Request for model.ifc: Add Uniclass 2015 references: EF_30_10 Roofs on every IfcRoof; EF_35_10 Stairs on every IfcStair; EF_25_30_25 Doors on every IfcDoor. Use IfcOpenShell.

First a look at what the model holds.

```python
import ifcopenshell

model = ifcopenshell.open("model.ifc")
print(model.schema)
print("classifications:", [c.Name for c in model.by_type("IfcClassification")])
for ifc_class in ("IfcDoor", "IfcRoof", "IfcStair", "IfcWall", "IfcWindow"):
    print(ifc_class, len(model.by_type(ifc_class)))
```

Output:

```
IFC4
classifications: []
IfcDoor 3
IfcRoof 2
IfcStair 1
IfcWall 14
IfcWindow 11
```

```python
import ifcopenshell
import ifcopenshell.api.classification

model = ifcopenshell.open("model.ifc")

system = ifcopenshell.api.classification.add_classification(model, classification="Uniclass 2015")

codes = {
    "IfcRoof": ("EF_30_10", "Roofs"),
    "IfcStair": ("EF_35_10", "Stairs"),
    "IfcDoor": ("EF_25_30_25", "Doors"),
}
for ifc_class, (code, name) in codes.items():
    products = model.by_type(ifc_class)
    ifcopenshell.api.classification.add_reference(
        model, products=products, classification=system, identification=code, name=name
    )
    print(code, len(products))

model.write("model-out.ifc")
```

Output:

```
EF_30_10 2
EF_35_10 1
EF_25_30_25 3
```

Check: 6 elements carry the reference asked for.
